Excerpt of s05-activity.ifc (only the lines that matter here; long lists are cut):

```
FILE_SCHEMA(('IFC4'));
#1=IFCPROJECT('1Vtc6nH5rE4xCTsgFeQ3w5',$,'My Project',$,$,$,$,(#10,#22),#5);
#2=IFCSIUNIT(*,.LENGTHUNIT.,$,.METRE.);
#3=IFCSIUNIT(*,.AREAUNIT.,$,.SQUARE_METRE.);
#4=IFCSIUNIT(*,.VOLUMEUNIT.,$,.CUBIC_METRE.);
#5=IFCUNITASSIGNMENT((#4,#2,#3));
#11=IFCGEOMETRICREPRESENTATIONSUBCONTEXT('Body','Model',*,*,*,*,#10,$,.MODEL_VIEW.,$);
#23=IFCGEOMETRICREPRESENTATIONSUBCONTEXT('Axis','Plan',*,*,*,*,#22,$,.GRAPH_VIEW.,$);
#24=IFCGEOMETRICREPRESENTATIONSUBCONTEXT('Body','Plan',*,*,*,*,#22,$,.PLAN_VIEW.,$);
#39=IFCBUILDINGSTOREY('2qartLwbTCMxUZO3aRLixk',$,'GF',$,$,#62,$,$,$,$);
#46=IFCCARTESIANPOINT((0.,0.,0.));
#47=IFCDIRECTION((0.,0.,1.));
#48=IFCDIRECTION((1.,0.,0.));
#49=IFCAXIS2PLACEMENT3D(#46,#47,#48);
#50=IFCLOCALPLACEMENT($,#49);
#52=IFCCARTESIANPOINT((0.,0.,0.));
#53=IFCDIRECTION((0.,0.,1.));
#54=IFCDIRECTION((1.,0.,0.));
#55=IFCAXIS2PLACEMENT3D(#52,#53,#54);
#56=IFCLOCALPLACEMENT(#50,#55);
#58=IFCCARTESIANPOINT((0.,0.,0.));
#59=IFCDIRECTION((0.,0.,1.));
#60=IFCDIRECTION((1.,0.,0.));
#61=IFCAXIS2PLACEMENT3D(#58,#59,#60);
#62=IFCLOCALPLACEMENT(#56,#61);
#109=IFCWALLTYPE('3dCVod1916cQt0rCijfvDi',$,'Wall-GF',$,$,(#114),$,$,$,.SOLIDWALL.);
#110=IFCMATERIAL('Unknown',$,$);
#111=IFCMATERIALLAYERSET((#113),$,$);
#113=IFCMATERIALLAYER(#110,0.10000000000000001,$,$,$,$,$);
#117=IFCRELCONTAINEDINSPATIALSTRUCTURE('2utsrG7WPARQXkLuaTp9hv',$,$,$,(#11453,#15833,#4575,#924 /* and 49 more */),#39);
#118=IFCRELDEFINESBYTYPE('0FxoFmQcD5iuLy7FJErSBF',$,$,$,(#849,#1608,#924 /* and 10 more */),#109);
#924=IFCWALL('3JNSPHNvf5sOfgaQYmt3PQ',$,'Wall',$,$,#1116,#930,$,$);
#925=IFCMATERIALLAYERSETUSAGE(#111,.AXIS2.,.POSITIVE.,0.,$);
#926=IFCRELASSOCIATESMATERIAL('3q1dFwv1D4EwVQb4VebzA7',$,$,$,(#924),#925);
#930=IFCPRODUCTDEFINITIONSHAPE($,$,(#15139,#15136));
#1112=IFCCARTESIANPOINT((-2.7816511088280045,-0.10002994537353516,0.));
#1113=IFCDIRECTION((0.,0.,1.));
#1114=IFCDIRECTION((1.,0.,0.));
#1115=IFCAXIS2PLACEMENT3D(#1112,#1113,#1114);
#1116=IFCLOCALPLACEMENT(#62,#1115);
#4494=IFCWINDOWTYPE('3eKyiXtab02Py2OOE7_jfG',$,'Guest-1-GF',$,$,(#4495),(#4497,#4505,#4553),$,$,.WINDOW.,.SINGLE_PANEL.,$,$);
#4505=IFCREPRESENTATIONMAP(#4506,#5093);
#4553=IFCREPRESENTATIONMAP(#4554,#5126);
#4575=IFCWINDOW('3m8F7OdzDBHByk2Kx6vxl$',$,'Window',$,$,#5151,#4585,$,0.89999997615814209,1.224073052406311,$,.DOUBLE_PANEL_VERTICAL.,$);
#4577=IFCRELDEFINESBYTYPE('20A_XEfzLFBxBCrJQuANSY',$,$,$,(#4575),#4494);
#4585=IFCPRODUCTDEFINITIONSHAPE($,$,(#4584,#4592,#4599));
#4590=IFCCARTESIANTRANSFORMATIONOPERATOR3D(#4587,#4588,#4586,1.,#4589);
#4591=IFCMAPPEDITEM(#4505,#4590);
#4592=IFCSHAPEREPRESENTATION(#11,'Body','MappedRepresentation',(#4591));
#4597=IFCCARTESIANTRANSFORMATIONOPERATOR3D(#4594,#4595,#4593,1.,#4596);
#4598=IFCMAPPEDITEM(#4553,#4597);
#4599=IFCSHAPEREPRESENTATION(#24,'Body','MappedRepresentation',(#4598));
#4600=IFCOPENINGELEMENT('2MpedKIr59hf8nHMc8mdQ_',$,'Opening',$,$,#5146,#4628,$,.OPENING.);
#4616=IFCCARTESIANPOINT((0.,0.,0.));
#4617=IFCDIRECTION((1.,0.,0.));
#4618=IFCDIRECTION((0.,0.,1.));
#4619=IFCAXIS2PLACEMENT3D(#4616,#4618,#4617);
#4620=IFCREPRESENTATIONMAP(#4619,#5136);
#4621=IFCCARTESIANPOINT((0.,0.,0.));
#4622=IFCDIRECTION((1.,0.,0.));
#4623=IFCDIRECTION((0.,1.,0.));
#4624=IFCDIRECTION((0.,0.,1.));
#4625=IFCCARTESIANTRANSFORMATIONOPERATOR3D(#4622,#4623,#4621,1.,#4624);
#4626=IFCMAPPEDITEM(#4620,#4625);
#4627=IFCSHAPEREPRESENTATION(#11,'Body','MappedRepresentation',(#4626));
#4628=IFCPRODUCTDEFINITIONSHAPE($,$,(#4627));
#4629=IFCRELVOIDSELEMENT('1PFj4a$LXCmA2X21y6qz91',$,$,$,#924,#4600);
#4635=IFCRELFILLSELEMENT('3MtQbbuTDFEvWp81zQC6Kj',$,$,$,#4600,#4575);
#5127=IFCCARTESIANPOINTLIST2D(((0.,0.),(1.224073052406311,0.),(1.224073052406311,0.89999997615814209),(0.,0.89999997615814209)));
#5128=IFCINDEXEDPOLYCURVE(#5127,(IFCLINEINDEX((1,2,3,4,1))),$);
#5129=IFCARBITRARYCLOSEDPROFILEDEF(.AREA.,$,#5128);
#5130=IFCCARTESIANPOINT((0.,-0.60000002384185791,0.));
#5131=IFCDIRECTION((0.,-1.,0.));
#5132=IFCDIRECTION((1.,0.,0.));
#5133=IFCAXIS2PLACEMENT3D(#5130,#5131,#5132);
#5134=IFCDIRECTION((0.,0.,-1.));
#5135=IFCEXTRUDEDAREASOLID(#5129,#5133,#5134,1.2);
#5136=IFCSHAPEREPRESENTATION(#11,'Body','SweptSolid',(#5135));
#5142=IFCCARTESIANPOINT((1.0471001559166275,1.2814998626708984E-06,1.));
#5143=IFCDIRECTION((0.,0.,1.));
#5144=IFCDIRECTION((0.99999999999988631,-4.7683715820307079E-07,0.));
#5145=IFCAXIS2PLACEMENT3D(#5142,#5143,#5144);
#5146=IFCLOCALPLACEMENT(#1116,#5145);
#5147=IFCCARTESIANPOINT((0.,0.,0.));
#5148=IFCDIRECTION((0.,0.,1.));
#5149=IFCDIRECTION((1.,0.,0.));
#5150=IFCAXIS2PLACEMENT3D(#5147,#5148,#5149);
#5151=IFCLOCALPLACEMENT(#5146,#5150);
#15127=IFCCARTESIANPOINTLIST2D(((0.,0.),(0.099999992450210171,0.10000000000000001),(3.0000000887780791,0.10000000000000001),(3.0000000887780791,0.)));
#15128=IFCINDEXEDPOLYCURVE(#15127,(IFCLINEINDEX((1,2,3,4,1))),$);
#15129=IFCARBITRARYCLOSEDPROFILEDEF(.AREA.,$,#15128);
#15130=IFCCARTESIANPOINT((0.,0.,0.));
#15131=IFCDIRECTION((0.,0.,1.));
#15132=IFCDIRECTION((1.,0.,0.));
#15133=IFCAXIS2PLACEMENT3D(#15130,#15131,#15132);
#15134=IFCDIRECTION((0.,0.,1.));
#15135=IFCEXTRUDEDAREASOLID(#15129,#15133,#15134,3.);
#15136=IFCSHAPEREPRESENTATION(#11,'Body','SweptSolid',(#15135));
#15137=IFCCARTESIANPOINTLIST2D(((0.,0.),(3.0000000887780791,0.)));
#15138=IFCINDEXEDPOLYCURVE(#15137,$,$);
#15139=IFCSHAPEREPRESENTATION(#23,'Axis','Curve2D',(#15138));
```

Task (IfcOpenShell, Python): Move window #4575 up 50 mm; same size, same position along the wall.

```python
import numpy as np
import ifcopenshell
import ifcopenshell.api.geometry
import ifcopenshell.util.placement
import ifcopenshell.util.unit

model = ifcopenshell.open("s05-activity.ifc")
unit_scale = ifcopenshell.util.unit.calculate_unit_scale(model)

window = model.by_guid("3m8F7OdzDBHByk2Kx6vxl$")
opening = window.FillsVoids[0].RelatingOpeningElement
dz = 0.05 / unit_scale

shift = np.array([0.0, 0.0, dz])
# The window is placed relative to its opening, so it follows when the opening moves.
matrix = ifcopenshell.util.placement.get_local_placement(opening.ObjectPlacement)
matrix[:3, 3] += shift
ifcopenshell.api.geometry.edit_object_placement(
    model, product=opening, matrix=matrix, is_si=False, should_transform_children=True
)

print(f"moved by {dz * unit_scale:+.3f} m")

model.write("s05-activity-out.ifc")
```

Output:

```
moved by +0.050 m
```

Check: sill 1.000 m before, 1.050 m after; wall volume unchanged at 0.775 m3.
